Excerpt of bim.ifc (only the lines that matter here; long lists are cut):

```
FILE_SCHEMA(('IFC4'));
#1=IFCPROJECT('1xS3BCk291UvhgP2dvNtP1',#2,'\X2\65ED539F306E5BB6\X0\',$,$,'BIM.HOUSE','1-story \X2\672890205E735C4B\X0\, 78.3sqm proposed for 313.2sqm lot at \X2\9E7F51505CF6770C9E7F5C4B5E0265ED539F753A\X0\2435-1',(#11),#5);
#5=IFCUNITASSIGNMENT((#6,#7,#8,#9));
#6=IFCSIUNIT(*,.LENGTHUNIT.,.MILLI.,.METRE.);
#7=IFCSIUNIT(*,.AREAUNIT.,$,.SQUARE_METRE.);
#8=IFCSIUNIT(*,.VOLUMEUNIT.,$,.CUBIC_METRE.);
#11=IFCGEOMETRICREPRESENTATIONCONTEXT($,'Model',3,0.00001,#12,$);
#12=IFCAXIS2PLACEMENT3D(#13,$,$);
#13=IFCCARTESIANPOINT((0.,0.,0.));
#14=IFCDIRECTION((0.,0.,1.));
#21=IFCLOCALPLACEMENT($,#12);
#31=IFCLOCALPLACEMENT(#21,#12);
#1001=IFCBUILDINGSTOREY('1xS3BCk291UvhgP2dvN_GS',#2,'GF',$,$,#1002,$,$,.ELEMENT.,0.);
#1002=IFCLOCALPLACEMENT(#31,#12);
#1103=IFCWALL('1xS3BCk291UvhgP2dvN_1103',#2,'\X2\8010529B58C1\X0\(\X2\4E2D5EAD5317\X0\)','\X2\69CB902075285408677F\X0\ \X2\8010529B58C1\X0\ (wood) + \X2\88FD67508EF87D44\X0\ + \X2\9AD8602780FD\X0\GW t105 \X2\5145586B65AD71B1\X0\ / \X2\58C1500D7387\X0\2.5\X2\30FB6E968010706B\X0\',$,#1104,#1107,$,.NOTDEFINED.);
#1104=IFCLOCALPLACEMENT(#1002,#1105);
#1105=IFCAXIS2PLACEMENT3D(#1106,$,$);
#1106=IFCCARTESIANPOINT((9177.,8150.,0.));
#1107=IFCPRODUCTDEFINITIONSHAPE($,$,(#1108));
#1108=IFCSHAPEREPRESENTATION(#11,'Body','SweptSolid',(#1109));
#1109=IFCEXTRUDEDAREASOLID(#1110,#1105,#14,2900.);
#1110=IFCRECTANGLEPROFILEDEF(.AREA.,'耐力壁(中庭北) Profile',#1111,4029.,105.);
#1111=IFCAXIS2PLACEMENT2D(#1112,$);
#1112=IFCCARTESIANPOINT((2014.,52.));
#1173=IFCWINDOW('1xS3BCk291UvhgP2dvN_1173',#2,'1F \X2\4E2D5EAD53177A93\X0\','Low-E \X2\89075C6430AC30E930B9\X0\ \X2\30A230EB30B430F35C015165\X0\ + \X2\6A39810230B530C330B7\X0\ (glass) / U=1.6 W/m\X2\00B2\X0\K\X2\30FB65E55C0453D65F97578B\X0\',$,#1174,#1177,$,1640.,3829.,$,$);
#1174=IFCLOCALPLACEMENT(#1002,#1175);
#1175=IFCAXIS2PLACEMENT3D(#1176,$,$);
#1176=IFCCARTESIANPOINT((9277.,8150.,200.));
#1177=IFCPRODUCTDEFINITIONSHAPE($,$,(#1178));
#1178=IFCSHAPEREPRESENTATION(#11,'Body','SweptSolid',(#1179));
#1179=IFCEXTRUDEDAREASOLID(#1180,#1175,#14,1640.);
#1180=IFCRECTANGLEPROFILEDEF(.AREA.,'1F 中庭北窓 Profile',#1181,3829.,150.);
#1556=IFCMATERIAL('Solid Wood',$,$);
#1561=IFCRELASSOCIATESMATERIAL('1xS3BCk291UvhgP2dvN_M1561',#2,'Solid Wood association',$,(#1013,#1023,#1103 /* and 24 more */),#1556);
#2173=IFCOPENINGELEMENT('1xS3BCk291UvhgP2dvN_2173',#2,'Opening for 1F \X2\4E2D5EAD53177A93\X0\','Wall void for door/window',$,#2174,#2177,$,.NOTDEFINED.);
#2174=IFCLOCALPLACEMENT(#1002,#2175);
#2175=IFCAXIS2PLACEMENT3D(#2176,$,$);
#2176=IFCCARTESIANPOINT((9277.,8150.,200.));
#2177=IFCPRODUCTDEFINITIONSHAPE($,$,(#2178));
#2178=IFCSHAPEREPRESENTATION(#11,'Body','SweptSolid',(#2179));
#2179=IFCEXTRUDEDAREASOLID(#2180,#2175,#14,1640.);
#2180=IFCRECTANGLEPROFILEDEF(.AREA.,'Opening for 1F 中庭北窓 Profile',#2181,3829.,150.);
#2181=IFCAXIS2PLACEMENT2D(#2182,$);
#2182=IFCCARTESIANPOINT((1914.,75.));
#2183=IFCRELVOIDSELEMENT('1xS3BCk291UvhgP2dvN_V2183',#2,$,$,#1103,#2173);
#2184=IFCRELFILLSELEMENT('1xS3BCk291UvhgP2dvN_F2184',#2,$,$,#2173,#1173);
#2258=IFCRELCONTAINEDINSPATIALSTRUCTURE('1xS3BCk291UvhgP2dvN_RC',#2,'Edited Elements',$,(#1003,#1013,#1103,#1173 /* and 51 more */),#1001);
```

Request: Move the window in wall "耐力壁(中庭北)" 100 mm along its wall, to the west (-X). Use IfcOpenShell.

```python
import ifcopenshell
import ifcopenshell.api.geometry
import ifcopenshell.util.placement
import ifcopenshell.util.unit

model = ifcopenshell.open("bim.ifc")
unit_scale = ifcopenshell.util.unit.calculate_unit_scale(model)

window = model.by_id(1173)
opening = window.FillsVoids[0].RelatingOpeningElement
wall = opening.VoidsElements[0].RelatingBuildingElement

wall_matrix = ifcopenshell.util.placement.get_local_placement(wall.ObjectPlacement)
shift = wall_matrix[:3, 0] * -0.1 / unit_scale
before = ifcopenshell.util.placement.get_local_placement(window.ObjectPlacement)[:3, 3].copy()

# The window is not placed relative to its opening, so move both.
for product in (opening, window):
    matrix = ifcopenshell.util.placement.get_local_placement(product.ObjectPlacement)
    matrix[:3, 3] += shift
    ifcopenshell.api.geometry.edit_object_placement(model, product=product, matrix=matrix, is_si=False)

after = ifcopenshell.util.placement.get_local_placement(window.ObjectPlacement)[:3, 3]
print("window moved by", (after - before).round(3) + 0.0)

model.write("bim-out.ifc")
```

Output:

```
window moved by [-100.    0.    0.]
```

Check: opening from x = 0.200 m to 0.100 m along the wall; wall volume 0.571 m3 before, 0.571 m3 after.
